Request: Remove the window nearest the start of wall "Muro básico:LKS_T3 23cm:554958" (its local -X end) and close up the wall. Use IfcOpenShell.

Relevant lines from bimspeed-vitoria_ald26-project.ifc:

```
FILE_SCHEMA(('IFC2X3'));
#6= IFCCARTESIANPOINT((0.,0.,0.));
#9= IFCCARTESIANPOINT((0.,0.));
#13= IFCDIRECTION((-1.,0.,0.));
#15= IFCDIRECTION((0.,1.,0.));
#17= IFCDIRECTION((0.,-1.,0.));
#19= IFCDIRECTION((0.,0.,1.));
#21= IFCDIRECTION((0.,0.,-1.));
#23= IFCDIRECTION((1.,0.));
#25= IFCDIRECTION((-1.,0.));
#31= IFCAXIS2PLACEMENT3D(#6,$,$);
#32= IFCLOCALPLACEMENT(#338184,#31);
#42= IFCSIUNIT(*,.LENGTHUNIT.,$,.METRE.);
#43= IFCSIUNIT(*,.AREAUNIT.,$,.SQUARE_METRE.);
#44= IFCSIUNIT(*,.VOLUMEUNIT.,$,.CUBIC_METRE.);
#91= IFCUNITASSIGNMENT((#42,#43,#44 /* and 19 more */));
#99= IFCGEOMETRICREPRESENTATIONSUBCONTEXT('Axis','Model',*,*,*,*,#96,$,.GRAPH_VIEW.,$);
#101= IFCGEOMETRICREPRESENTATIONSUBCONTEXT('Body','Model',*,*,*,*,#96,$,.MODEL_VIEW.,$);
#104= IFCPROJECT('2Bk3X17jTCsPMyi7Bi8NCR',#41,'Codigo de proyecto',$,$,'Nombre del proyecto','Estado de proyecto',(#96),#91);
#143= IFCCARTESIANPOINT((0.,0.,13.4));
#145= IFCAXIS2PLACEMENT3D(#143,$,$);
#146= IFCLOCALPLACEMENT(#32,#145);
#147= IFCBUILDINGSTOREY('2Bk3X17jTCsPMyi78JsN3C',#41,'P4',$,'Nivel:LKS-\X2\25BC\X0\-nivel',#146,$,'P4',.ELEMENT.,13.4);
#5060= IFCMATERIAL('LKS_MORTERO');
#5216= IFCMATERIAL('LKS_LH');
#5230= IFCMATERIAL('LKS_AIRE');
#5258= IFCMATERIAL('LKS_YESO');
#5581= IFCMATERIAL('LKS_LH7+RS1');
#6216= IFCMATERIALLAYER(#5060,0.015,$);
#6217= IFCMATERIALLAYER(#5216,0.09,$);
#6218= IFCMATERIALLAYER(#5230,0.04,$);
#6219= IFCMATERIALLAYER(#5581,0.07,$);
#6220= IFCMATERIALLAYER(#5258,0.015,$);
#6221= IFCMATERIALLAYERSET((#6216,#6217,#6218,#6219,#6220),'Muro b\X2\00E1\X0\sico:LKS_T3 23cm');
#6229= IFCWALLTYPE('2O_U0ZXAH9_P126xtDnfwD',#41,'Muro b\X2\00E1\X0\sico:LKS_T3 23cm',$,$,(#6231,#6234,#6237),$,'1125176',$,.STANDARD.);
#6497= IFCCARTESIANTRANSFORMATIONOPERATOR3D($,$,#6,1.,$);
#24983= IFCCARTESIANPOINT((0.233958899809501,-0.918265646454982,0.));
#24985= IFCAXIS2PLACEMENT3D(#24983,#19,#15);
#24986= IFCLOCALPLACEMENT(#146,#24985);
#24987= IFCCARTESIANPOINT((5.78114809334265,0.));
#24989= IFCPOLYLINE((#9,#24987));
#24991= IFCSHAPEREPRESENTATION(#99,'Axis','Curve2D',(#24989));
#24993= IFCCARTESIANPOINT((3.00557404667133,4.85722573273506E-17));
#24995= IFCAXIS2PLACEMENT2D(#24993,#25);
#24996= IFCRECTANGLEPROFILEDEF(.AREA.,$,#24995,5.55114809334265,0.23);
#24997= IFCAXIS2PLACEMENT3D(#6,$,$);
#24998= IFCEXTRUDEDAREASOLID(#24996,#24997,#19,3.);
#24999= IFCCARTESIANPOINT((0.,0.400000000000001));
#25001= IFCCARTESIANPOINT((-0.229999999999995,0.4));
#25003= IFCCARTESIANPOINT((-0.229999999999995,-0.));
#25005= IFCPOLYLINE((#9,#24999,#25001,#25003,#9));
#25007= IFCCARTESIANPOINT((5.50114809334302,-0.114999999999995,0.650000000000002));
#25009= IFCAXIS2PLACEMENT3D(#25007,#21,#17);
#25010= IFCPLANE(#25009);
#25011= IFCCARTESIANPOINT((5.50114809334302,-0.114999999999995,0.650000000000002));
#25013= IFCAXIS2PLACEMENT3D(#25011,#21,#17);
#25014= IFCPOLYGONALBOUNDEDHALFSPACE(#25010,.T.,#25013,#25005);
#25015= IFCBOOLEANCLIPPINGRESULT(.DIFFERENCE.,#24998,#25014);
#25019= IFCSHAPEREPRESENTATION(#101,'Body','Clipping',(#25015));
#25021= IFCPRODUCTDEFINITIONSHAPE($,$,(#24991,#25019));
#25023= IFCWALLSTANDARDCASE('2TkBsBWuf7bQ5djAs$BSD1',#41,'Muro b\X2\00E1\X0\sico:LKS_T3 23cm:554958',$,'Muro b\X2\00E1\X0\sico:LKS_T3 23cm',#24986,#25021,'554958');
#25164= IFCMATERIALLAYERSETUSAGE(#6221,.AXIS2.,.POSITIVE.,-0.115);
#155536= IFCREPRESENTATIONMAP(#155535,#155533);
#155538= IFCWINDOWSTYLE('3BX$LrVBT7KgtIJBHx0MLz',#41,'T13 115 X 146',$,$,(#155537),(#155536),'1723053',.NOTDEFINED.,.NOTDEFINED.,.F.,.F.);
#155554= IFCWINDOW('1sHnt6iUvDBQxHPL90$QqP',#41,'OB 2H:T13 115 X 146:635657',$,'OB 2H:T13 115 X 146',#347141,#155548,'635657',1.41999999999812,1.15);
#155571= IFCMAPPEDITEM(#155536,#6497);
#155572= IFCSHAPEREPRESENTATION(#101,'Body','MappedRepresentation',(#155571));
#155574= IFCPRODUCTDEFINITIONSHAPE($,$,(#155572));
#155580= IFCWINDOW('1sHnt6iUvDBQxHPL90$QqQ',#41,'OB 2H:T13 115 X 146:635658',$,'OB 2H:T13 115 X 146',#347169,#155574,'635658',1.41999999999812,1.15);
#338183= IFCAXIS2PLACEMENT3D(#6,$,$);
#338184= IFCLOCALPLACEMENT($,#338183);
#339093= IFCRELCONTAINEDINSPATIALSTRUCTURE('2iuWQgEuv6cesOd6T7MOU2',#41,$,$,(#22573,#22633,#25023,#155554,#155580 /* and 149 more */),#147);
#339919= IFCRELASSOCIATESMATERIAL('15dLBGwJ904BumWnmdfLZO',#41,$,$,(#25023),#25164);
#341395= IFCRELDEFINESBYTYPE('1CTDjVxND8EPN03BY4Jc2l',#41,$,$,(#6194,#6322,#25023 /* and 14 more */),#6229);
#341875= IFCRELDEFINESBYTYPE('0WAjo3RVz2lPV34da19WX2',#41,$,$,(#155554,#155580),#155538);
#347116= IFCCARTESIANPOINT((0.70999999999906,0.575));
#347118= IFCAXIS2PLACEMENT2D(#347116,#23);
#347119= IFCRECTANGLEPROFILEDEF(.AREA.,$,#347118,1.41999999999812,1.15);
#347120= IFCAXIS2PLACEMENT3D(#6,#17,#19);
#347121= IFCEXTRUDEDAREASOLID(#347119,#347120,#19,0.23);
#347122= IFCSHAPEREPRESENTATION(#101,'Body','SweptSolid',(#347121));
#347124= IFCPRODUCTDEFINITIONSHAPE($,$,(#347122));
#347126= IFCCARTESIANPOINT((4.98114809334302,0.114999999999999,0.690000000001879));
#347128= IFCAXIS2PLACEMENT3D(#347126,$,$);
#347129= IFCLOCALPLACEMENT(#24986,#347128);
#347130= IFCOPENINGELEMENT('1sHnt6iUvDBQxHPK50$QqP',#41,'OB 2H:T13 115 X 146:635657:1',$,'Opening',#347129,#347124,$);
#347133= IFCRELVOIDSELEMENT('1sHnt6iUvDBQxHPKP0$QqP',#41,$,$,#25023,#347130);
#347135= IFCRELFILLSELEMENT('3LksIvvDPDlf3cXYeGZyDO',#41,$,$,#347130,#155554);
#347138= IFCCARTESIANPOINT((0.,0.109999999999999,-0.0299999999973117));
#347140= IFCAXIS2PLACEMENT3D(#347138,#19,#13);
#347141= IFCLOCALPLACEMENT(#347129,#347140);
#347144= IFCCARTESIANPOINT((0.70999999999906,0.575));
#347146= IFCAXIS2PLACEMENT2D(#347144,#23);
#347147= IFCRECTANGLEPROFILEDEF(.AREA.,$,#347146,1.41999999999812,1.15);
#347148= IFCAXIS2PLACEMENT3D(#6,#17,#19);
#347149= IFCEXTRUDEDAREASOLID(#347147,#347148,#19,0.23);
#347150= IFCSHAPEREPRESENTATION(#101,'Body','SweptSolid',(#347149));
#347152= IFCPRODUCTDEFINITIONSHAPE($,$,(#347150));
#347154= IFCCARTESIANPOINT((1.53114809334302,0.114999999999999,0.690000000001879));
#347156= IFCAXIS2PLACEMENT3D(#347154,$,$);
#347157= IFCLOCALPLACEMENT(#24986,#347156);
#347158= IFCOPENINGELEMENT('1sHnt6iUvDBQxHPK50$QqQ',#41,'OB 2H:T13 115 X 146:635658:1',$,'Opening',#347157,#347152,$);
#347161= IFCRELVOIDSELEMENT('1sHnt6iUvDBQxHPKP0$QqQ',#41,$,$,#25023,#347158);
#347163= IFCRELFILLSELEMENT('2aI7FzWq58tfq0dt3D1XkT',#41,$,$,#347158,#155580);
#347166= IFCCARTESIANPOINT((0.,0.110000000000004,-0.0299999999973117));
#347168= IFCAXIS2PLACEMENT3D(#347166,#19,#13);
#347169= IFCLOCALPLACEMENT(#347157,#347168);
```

```python
import ifcopenshell
import ifcopenshell.api.feature
import ifcopenshell.api.root
import ifcopenshell.geom
import ifcopenshell.util.shape

model = ifcopenshell.open("bimspeed-vitoria_ald26-project.ifc")
settings = ifcopenshell.geom.settings()


def volume(element):
    """Net volume in cubic metres, openings subtracted."""
    shape = ifcopenshell.geom.create_shape(settings, element)
    return ifcopenshell.util.shape.get_volume(shape.geometry)


window = model.by_guid("1sHnt6iUvDBQxHPL90$QqQ")
opening = window.FillsVoids[0].RelatingOpeningElement
wall = opening.VoidsElements[0].RelatingBuildingElement
before = volume(wall)

ifcopenshell.api.root.remove_product(model, product=window)
ifcopenshell.api.feature.remove_feature(model, feature=opening)

after = volume(wall)

print(f"wall volume {before:.3f} -> {after:.3f} m3")

model.write("bimspeed-vitoria_ald26-project_rev.ifc")
```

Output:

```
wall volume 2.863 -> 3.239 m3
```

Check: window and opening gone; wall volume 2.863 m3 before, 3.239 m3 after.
